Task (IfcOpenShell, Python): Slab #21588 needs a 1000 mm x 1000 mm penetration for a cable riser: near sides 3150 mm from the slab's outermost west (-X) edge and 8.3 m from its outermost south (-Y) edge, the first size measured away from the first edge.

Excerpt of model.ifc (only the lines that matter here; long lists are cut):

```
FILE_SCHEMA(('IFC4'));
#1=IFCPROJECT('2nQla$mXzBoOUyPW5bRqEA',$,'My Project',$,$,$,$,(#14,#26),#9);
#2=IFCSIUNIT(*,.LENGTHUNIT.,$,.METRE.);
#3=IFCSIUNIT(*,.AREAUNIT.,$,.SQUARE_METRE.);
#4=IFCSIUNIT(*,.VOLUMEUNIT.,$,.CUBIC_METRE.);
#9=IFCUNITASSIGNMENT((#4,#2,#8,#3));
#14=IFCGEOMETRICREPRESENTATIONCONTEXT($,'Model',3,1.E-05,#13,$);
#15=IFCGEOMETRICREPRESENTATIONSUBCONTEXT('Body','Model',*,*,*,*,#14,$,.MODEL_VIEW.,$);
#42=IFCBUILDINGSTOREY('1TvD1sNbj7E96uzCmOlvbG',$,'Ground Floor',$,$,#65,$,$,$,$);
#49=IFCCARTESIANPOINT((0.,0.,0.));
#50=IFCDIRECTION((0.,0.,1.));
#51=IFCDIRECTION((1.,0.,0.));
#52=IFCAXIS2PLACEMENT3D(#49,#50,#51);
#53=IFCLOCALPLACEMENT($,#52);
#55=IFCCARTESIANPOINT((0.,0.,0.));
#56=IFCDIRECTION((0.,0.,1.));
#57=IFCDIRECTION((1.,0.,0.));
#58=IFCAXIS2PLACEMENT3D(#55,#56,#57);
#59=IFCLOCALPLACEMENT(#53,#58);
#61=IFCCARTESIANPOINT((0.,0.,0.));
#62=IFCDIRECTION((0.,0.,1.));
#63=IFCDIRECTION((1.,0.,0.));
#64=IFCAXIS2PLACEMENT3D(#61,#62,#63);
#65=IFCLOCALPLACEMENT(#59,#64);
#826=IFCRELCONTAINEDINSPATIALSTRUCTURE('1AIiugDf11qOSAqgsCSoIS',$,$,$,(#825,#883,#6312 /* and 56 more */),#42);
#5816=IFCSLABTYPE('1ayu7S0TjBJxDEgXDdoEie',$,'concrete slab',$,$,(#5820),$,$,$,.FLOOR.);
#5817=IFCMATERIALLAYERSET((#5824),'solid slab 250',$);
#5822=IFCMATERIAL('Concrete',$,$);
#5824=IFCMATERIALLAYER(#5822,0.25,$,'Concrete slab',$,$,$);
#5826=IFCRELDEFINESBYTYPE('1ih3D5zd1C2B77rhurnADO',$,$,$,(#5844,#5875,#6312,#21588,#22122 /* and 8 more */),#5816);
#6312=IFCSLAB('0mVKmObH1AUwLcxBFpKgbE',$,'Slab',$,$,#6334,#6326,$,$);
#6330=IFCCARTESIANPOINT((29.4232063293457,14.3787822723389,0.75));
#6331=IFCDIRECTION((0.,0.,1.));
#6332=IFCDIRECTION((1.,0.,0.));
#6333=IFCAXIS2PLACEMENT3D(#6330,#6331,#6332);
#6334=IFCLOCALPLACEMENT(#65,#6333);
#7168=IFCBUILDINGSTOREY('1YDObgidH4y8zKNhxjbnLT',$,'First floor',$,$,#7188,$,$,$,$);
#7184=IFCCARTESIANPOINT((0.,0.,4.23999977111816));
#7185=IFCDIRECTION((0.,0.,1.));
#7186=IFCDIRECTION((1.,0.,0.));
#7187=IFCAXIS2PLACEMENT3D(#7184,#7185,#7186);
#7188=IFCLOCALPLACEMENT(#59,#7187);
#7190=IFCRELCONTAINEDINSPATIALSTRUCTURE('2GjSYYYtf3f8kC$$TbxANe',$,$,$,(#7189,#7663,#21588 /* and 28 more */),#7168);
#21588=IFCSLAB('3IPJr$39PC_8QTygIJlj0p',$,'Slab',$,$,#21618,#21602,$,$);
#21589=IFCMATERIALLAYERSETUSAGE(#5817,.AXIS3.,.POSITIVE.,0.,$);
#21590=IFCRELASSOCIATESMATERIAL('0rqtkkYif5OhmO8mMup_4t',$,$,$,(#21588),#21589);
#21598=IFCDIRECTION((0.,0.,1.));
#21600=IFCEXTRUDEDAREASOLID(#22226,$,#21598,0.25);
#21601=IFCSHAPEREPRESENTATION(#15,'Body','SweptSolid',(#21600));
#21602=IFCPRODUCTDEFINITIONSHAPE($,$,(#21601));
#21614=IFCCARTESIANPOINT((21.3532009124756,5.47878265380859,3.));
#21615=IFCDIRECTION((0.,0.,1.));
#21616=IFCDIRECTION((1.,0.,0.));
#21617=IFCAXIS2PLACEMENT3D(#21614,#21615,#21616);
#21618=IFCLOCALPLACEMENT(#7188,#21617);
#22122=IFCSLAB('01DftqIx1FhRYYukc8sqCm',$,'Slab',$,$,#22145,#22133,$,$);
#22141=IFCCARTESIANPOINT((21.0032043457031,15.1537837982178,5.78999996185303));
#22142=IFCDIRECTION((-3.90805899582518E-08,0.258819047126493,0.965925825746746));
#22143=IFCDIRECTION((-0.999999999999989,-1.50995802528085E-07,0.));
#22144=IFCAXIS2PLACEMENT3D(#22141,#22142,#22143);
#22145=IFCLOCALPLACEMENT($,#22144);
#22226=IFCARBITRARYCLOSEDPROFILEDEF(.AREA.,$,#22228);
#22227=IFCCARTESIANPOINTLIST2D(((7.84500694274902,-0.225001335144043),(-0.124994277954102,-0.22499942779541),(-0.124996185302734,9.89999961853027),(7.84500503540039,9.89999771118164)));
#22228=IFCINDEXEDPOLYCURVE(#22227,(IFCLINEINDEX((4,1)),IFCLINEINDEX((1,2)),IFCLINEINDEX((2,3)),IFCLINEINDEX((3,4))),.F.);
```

```python
import numpy as np
import ifcopenshell
import ifcopenshell.api.feature
import ifcopenshell.api.geometry
import ifcopenshell.api.root
import ifcopenshell.geom
import ifcopenshell.util.placement
import ifcopenshell.util.representation
import ifcopenshell.util.shape
import ifcopenshell.util.unit

model = ifcopenshell.open("model.ifc")
unit_scale = ifcopenshell.util.unit.calculate_unit_scale(model)
settings = ifcopenshell.geom.settings()


def volume(element):
    """Net volume in cubic metres, openings subtracted."""
    shape = ifcopenshell.geom.create_shape(settings, element)
    return ifcopenshell.util.shape.get_volume(shape.geometry)


slab = model.by_guid("3IPJr$39PC_8QTygIJlj0p")
before = volume(slab)

# Extent in the slab's own axes, in metres. The edges named are its -X and -Y sides.
slab_shape = ifcopenshell.geom.create_shape(settings, slab)
vertices = ifcopenshell.util.shape.get_vertices(slab_shape.geometry)
x_min, y_min, bottom = vertices.min(axis=0)
top = vertices[:, 2].max()

opening = ifcopenshell.api.root.create_entity(model, ifc_class="IfcOpeningElement", name="Cable riser opening", predefined_type="OPENING")
context = ifcopenshell.util.representation.get_context(model, "Model", "Body", "MODEL_VIEW")
width, depth = 1, 1
outline = [(0.0, 0.0), (width, 0.0), (width, depth), (0.0, depth), (0.0, 0.0)]
# Overshoot both faces by 50 mm so the cut is clean.
shape = ifcopenshell.api.geometry.add_slab_representation(
    model, context=context, depth=top - bottom + 0.1, polyline=outline
)
ifcopenshell.api.geometry.assign_representation(model, product=opening, representation=shape)

matrix = ifcopenshell.util.placement.get_local_placement(slab.ObjectPlacement)
matrix[:, 3] = matrix @ np.append(np.array([x_min + 3.15, y_min + 8.3, bottom - 0.05]) / unit_scale, 1.0)
ifcopenshell.api.geometry.edit_object_placement(model, product=opening, matrix=matrix, is_si=False)
ifcopenshell.api.feature.add_feature(model, feature=opening, element=slab)

after = volume(slab)

print(f"slab volume {before:.3f} -> {after:.3f} m3")

model.write("model-out.ifc")
```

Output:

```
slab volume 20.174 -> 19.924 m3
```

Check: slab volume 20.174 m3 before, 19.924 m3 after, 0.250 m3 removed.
